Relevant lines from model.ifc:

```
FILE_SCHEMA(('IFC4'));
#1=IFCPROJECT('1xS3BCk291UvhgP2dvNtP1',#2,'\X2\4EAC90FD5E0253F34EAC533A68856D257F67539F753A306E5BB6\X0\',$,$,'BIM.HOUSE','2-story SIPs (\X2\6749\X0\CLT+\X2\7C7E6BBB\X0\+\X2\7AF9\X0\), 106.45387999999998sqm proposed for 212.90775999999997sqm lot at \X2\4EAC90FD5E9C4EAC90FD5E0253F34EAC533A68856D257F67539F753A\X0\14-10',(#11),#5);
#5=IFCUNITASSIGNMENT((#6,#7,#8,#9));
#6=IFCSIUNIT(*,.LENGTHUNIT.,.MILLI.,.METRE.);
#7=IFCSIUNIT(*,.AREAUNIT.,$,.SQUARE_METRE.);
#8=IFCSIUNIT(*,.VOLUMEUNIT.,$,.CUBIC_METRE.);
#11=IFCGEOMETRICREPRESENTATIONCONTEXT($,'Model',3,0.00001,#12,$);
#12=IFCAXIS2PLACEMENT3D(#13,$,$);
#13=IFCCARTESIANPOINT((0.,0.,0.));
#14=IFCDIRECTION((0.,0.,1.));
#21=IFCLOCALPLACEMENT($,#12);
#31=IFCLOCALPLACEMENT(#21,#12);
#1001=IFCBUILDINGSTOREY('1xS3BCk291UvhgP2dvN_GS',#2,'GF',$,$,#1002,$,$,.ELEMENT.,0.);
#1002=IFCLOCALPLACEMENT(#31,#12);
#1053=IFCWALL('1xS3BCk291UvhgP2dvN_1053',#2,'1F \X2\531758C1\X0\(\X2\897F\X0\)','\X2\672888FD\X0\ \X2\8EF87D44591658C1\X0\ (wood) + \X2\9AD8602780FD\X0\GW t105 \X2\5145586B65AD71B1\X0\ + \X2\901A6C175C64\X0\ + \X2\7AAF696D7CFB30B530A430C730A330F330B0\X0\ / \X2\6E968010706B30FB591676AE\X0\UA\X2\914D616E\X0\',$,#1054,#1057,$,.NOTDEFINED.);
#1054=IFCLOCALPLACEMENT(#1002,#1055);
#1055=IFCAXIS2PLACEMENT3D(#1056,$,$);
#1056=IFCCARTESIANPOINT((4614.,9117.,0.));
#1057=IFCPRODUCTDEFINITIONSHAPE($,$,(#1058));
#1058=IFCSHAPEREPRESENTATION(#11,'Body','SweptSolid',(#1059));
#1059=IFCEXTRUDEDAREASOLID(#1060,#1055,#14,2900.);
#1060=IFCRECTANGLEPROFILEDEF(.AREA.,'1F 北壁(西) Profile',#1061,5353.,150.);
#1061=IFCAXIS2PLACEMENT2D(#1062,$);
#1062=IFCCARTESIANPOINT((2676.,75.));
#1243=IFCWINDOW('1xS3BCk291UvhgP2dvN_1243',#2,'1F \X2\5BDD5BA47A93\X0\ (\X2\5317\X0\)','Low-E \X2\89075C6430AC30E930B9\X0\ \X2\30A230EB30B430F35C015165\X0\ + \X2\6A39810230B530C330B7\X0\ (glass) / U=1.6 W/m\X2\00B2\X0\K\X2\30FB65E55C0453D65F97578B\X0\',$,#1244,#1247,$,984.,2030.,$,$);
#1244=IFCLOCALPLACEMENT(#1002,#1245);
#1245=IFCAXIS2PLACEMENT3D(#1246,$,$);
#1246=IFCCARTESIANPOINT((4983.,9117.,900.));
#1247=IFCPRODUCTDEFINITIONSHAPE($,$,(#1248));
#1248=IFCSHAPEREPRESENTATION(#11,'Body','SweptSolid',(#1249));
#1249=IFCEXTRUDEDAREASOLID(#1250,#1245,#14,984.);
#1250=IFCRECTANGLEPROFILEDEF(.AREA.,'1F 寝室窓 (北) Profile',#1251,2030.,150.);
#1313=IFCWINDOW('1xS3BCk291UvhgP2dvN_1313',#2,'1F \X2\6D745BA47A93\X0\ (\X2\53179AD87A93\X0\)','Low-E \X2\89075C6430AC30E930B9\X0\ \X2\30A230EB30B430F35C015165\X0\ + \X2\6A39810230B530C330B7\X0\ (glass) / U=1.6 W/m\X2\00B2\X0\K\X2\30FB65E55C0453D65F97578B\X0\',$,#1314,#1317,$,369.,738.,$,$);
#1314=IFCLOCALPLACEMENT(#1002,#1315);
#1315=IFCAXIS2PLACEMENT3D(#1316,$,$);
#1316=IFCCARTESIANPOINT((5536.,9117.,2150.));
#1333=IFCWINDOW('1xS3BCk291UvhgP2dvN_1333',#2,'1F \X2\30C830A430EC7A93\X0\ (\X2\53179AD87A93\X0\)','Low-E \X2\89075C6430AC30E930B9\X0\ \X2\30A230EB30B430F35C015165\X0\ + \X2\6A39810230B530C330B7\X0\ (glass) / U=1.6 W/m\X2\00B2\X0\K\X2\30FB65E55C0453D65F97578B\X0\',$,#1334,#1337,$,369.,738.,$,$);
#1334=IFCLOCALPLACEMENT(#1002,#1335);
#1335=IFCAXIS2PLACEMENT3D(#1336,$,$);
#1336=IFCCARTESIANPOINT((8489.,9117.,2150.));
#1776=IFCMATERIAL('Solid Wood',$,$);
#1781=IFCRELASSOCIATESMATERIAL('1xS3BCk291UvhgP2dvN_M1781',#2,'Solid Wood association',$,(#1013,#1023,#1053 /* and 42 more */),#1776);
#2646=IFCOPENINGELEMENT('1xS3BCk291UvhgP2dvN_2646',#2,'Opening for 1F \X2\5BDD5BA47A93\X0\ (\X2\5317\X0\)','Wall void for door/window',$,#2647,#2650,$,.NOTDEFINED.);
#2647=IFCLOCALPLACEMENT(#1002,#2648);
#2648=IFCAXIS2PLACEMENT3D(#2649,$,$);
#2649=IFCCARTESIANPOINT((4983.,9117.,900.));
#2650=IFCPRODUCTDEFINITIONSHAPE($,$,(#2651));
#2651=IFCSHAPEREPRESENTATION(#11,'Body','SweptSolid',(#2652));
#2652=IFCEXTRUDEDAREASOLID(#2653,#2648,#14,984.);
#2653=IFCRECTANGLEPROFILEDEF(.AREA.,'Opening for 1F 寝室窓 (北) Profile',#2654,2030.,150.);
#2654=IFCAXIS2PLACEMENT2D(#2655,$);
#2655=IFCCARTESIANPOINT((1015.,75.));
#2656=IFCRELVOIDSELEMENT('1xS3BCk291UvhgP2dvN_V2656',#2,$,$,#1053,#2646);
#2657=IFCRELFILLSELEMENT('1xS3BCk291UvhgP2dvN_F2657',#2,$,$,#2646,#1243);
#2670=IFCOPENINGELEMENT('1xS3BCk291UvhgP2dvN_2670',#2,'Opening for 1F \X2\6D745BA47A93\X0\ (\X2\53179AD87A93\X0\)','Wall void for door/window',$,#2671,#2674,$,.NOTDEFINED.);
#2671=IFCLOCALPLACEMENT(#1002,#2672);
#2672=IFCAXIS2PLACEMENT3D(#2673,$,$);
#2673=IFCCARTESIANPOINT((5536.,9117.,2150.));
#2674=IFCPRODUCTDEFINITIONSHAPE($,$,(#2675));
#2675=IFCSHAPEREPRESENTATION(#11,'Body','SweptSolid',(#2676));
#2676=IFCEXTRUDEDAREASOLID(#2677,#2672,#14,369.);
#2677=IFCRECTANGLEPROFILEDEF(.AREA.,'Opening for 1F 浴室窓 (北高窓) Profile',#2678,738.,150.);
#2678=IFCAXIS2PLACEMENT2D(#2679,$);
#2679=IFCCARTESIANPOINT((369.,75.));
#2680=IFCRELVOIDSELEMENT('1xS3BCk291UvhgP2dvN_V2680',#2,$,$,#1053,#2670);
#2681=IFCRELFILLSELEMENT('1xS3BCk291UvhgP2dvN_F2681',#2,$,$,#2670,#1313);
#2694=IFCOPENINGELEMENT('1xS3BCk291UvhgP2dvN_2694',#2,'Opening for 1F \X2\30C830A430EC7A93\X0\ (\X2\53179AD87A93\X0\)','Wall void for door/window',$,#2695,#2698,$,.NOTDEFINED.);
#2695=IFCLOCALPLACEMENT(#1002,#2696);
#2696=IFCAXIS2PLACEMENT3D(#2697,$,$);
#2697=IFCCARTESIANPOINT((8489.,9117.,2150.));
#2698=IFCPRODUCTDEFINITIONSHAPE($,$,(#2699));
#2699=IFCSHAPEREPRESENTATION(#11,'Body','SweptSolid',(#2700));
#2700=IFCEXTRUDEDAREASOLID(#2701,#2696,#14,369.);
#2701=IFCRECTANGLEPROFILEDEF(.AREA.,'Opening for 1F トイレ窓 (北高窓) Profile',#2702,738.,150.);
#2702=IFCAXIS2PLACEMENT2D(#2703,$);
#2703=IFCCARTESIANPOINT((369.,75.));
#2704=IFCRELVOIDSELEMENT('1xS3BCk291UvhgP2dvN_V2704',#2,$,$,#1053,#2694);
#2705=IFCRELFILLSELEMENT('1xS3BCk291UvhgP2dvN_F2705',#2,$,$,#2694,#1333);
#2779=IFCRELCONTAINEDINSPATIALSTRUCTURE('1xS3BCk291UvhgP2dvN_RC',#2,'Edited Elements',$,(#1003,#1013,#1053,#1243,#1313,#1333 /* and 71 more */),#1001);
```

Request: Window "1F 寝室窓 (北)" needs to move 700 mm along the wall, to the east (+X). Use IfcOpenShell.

```python
import ifcopenshell
import ifcopenshell.api.geometry
import ifcopenshell.util.placement
import ifcopenshell.util.unit

model = ifcopenshell.open("model.ifc")
unit_scale = ifcopenshell.util.unit.calculate_unit_scale(model)

window = model.by_guid("1xS3BCk291UvhgP2dvN_1243")
opening = window.FillsVoids[0].RelatingOpeningElement
wall = opening.VoidsElements[0].RelatingBuildingElement

wall_matrix = ifcopenshell.util.placement.get_local_placement(wall.ObjectPlacement)
shift = wall_matrix[:3, 0] * 0.7 / unit_scale
before = ifcopenshell.util.placement.get_local_placement(window.ObjectPlacement)[:3, 3].copy()

# The window is not placed relative to its opening, so move both.
for product in (opening, window):
    matrix = ifcopenshell.util.placement.get_local_placement(product.ObjectPlacement)
    matrix[:3, 3] += shift
    ifcopenshell.api.geometry.edit_object_placement(model, product=product, matrix=matrix, is_si=False)

after = ifcopenshell.util.placement.get_local_placement(window.ObjectPlacement)[:3, 3]
print("window moved by", (after - before).round(3) + 0.0)

model.write("model_edited.ifc")
```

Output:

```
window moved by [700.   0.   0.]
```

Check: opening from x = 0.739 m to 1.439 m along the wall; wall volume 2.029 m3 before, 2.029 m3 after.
